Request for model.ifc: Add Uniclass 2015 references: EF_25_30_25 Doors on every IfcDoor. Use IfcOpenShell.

First a look at what the model holds.

```python
import ifcopenshell

model = ifcopenshell.open("model.ifc")
print(model.schema)
print("classifications:", [c.Name for c in model.by_type("IfcClassification")])
for ifc_class in ("IfcDoor", "IfcRoof", "IfcStair", "IfcWall", "IfcWindow"):
    print(ifc_class, len(model.by_type(ifc_class)))
```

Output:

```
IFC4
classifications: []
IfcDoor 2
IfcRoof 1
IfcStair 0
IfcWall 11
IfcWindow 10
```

```python
import ifcopenshell
import ifcopenshell.api.classification

model = ifcopenshell.open("model.ifc")

system = ifcopenshell.api.classification.add_classification(model, classification="Uniclass 2015")

codes = {
    "IfcDoor": ("EF_25_30_25", "Doors"),
}
for ifc_class, (code, name) in codes.items():
    products = model.by_type(ifc_class)
    ifcopenshell.api.classification.add_reference(
        model, products=products, classification=system, identification=code, name=name
    )
    print(code, len(products))

model.write("model_updated.ifc")
```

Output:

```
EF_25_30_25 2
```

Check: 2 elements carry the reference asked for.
